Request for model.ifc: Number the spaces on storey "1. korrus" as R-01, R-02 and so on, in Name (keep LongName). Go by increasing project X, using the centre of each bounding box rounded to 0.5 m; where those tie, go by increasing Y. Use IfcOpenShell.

First a look at what the model holds.

```python
import ifcopenshell
import ifcopenshell.util.element
import ifcopenshell.util.placement

model = ifcopenshell.open("model.ifc")
print(model.schema)
storey = next(s for s in model.by_type("IfcBuildingStorey") if s.Name == "1. korrus")
spaces = [e for e in ifcopenshell.util.element.get_decomposition(storey) if e.is_a("IfcSpace")]
for e in sorted(spaces, key=lambda e: e.id()):
    origin = ifcopenshell.util.placement.get_local_placement(e.ObjectPlacement)[:3, 3]
    print(e.id(), e.Name, e.LongName, origin.round(2) + 0.0, sep=" | ")
```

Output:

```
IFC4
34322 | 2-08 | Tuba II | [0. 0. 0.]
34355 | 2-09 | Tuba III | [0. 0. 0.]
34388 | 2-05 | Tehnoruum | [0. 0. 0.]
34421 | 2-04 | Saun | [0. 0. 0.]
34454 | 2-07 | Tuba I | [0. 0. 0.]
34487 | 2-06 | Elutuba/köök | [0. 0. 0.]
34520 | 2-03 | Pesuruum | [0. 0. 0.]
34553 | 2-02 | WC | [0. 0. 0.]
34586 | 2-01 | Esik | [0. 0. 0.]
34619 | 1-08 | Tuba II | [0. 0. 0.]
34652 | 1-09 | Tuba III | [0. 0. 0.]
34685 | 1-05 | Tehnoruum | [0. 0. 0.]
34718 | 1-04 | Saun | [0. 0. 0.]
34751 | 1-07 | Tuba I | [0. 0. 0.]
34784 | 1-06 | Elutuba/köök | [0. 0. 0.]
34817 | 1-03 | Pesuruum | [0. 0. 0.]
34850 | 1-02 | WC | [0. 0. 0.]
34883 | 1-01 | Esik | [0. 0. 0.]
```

```python
import ifcopenshell
import ifcopenshell.geom
import ifcopenshell.util.element
import ifcopenshell.util.shape

model = ifcopenshell.open("model.ifc")
settings = ifcopenshell.geom.settings()
settings.set("use-world-coords", True)


def centre(element):
    shape = ifcopenshell.geom.create_shape(settings, element)
    return ifcopenshell.util.shape.get_bbox_centroid(shape.geometry)


storey = next(s for s in model.by_type("IfcBuildingStorey") if s.Name == "1. korrus")
spaces = [e for e in ifcopenshell.util.element.get_decomposition(storey) if e.is_a("IfcSpace")]

# Insertion points can sit at a corner or the storey origin, so sort by the geometry (in metres).
centres = {e: centre(e) for e in spaces}
spaces.sort(key=lambda e: (round(centres[e][0] / 0.5), centres[e][1]))

for i, e in enumerate(spaces, start=1):
    number = f"R-{i:02d}"
    e.Name = number
    print(e.id(), number)

model.write("model_edited.ifc")
```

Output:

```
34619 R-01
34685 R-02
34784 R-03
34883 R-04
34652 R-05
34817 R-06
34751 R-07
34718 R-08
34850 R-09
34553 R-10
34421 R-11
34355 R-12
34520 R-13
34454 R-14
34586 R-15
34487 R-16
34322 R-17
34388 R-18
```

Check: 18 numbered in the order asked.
